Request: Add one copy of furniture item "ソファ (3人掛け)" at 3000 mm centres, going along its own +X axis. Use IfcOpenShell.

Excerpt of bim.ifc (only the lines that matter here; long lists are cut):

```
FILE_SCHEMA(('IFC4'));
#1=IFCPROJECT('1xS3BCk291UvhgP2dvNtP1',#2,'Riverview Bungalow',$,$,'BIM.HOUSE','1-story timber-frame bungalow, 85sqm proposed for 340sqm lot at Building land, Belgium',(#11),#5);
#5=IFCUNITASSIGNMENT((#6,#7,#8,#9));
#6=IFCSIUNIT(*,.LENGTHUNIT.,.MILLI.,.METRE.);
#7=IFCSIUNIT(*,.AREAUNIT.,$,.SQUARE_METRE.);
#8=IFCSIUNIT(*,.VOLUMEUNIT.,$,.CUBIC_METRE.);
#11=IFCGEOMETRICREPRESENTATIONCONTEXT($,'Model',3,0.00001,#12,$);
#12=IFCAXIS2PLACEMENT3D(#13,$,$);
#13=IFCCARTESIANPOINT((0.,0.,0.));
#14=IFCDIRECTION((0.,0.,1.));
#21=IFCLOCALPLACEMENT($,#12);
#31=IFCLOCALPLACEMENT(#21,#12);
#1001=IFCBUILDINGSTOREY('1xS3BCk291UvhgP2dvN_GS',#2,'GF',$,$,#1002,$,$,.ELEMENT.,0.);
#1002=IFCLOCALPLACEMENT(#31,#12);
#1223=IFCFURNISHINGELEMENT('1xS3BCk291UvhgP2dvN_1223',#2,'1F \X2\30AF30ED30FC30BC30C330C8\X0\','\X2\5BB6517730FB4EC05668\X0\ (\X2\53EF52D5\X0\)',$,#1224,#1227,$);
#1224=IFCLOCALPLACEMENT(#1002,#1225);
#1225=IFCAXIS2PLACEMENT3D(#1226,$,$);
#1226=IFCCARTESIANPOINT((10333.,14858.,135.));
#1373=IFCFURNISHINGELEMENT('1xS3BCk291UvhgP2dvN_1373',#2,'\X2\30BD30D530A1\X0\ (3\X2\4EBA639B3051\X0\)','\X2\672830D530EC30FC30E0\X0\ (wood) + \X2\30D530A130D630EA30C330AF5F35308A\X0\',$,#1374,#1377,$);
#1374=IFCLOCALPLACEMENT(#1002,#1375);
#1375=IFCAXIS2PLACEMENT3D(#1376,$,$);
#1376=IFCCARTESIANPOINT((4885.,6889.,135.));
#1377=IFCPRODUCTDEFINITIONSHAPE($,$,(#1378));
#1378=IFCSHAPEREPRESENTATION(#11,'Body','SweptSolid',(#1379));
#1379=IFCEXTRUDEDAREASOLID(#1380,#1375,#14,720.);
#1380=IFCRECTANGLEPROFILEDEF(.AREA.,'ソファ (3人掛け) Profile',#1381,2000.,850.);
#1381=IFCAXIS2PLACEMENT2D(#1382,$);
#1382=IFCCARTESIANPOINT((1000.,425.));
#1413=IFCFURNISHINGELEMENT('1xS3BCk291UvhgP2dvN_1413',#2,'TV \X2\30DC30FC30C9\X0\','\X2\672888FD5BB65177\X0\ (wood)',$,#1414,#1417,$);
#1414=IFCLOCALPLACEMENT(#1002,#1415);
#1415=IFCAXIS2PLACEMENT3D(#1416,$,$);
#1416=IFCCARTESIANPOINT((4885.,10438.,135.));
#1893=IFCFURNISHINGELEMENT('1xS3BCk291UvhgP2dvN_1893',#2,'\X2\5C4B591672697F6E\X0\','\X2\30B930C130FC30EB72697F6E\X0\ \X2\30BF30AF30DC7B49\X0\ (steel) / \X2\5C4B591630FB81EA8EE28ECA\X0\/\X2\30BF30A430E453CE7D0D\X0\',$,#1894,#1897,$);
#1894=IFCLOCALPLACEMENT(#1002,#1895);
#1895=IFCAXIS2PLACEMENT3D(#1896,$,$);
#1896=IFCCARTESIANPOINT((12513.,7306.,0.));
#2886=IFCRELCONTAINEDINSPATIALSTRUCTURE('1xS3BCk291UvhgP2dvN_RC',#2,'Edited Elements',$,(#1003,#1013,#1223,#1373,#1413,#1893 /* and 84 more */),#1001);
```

```python
import ifcopenshell
import ifcopenshell.api.geometry
import ifcopenshell.api.root
import ifcopenshell.util.element
import ifcopenshell.util.placement
import ifcopenshell.util.unit

model = ifcopenshell.open("bim.ifc")
unit_scale = ifcopenshell.util.unit.calculate_unit_scale(model)


def reuse_history(source, copy):
    """copy_class also copies each property set's owner history, people and application; keep the originals."""
    for rel in copy.IsDefinedBy:
        if rel.is_a("IfcRelDefinesByProperties") and (history := rel.RelatingPropertyDefinition.OwnerHistory):
            rel.RelatingPropertyDefinition.OwnerHistory = source.OwnerHistory
            ifcopenshell.util.element.remove_deep2(model, history)


source = model.by_guid("1xS3BCk291UvhgP2dvN_1373")
base = ifcopenshell.util.placement.get_local_placement(source.ObjectPlacement)
step = base[:3, 0] * 3 / unit_scale

for i in range(1, 2):
    copy = ifcopenshell.api.root.copy_class(model, product=source)
    copy.Representation = ifcopenshell.util.element.copy_deep(
        model, source.Representation, exclude=["IfcGeometricRepresentationContext", "IfcRepresentationMap"]
    )
    reuse_history(source, copy)
    matrix = base.copy()
    matrix[:3, 3] += i * step
    print("added at", matrix[:3, 3].round(3) + 0.0)
    ifcopenshell.api.geometry.edit_object_placement(model, product=copy, matrix=matrix, is_si=False)

model.write("bim_v2.ifc")
```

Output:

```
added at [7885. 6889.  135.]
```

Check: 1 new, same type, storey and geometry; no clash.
